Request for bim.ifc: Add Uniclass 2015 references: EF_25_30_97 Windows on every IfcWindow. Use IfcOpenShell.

First a look at what the model holds.

```python
import ifcopenshell

model = ifcopenshell.open("bim.ifc")
print(model.schema)
print("classifications:", [c.Name for c in model.by_type("IfcClassification")])
for ifc_class in ("IfcDoor", "IfcRoof", "IfcStair", "IfcWall", "IfcWindow"):
    print(ifc_class, len(model.by_type(ifc_class)))
```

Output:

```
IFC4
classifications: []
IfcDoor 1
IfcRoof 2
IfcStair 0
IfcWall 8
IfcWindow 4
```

```python
import ifcopenshell
import ifcopenshell.api.classification

model = ifcopenshell.open("bim.ifc")

system = ifcopenshell.api.classification.add_classification(model, classification="Uniclass 2015")

codes = {
    "IfcWindow": ("EF_25_30_97", "Windows"),
}
for ifc_class, (code, name) in codes.items():
    products = model.by_type(ifc_class)
    ifcopenshell.api.classification.add_reference(
        model, products=products, classification=system, identification=code, name=name
    )
    print(code, len(products))

model.write("bim_edited.ifc")
```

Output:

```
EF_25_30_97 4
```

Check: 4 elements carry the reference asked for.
